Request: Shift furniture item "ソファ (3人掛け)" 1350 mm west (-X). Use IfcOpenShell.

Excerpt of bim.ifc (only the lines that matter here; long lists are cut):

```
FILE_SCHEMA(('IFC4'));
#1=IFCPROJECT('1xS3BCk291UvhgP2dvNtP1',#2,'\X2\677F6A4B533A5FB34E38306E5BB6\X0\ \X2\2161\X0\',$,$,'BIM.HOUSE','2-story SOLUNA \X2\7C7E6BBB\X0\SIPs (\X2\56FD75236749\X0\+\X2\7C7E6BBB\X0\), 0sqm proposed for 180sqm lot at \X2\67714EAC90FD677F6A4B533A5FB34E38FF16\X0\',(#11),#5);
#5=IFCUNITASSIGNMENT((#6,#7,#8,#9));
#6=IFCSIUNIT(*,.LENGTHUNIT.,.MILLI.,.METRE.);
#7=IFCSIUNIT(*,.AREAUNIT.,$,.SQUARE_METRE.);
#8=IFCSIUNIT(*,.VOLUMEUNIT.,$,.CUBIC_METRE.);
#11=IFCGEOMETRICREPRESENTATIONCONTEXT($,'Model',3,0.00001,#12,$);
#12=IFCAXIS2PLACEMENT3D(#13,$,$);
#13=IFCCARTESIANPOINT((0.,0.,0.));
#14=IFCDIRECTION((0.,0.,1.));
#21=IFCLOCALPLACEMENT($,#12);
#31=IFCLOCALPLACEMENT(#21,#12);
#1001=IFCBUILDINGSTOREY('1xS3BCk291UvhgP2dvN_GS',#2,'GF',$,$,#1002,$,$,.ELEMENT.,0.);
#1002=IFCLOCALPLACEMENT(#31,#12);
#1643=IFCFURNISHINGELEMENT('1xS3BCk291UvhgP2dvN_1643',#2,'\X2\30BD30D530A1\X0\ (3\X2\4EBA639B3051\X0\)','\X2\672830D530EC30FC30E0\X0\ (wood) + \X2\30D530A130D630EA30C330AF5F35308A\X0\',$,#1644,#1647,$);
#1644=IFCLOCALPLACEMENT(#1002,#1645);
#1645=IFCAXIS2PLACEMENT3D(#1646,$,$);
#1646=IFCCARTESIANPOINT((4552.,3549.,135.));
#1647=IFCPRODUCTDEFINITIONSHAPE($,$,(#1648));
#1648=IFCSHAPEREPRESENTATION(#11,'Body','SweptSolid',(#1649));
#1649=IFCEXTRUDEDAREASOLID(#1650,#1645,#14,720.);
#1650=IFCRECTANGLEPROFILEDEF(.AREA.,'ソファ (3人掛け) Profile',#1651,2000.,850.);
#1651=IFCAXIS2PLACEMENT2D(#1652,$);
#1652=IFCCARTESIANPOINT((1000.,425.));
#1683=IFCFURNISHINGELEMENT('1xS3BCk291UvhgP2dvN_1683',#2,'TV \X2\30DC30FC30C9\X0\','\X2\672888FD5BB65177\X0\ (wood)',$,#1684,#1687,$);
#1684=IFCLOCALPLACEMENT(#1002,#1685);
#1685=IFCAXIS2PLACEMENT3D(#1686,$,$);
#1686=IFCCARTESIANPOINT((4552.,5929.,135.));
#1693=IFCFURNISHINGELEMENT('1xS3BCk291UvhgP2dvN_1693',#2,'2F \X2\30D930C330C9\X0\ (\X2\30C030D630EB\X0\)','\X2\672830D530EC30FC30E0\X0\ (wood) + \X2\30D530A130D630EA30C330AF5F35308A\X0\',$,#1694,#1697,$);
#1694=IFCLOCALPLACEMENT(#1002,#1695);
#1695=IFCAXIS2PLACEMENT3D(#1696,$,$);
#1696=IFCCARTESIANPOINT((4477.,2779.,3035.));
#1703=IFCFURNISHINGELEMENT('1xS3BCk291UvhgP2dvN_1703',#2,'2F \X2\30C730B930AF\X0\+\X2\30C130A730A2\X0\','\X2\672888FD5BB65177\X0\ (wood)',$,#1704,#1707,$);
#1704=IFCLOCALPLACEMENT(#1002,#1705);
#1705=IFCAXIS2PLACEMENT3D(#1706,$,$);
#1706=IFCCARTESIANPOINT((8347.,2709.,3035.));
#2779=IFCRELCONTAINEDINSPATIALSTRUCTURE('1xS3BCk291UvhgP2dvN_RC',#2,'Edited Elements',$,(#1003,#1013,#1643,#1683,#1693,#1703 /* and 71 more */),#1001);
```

```python
import ifcopenshell
import ifcopenshell.api.geometry
import ifcopenshell.util.placement
import ifcopenshell.util.unit

model = ifcopenshell.open("bim.ifc")
unit_scale = ifcopenshell.util.unit.calculate_unit_scale(model)

item = model.by_id(1643)
matrix = ifcopenshell.util.placement.get_local_placement(item.ObjectPlacement)
matrix[0, 3] -= 1.35 / unit_scale
ifcopenshell.api.geometry.edit_object_placement(model, product=item, matrix=matrix, is_si=False)

print(ifcopenshell.util.placement.get_local_placement(item.ObjectPlacement).round(3) + 0.0)

model.write("bim_v2.ifc")
```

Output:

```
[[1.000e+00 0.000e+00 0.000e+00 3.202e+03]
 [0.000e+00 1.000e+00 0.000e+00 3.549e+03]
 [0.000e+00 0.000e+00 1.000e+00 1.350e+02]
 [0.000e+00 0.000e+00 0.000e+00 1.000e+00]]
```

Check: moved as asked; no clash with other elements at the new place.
